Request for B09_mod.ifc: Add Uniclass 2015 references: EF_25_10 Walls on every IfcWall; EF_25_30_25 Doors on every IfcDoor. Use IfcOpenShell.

First a look at what the model holds.

```python
import ifcopenshell

model = ifcopenshell.open("B09_mod.ifc")
print(model.schema)
print("classifications:", [c.Name for c in model.by_type("IfcClassification")])
for ifc_class in ("IfcDoor", "IfcRoof", "IfcStair", "IfcWall", "IfcWindow"):
    print(ifc_class, len(model.by_type(ifc_class)))
```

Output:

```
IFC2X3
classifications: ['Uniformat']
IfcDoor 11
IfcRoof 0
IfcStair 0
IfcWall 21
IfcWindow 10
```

```python
import ifcopenshell
import ifcopenshell.api.classification

model = ifcopenshell.open("B09_mod.ifc")

# IFC2X3 requires Source and Edition and has no link from the project to the system.
system = model.create_entity("IfcClassification", Source="NBS", Edition="2015", Name="Uniclass 2015")

codes = {
    "IfcWall": ("EF_25_10", "Walls"),
    "IfcDoor": ("EF_25_30_25", "Doors"),
}
for ifc_class, (code, name) in codes.items():
    products = model.by_type(ifc_class)
    ifcopenshell.api.classification.add_reference(
        model, products=products, classification=system, identification=code, name=name
    )
    print(code, len(products))

model.write("B09_mod-out.ifc")
```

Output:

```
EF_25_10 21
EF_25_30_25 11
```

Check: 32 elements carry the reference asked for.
